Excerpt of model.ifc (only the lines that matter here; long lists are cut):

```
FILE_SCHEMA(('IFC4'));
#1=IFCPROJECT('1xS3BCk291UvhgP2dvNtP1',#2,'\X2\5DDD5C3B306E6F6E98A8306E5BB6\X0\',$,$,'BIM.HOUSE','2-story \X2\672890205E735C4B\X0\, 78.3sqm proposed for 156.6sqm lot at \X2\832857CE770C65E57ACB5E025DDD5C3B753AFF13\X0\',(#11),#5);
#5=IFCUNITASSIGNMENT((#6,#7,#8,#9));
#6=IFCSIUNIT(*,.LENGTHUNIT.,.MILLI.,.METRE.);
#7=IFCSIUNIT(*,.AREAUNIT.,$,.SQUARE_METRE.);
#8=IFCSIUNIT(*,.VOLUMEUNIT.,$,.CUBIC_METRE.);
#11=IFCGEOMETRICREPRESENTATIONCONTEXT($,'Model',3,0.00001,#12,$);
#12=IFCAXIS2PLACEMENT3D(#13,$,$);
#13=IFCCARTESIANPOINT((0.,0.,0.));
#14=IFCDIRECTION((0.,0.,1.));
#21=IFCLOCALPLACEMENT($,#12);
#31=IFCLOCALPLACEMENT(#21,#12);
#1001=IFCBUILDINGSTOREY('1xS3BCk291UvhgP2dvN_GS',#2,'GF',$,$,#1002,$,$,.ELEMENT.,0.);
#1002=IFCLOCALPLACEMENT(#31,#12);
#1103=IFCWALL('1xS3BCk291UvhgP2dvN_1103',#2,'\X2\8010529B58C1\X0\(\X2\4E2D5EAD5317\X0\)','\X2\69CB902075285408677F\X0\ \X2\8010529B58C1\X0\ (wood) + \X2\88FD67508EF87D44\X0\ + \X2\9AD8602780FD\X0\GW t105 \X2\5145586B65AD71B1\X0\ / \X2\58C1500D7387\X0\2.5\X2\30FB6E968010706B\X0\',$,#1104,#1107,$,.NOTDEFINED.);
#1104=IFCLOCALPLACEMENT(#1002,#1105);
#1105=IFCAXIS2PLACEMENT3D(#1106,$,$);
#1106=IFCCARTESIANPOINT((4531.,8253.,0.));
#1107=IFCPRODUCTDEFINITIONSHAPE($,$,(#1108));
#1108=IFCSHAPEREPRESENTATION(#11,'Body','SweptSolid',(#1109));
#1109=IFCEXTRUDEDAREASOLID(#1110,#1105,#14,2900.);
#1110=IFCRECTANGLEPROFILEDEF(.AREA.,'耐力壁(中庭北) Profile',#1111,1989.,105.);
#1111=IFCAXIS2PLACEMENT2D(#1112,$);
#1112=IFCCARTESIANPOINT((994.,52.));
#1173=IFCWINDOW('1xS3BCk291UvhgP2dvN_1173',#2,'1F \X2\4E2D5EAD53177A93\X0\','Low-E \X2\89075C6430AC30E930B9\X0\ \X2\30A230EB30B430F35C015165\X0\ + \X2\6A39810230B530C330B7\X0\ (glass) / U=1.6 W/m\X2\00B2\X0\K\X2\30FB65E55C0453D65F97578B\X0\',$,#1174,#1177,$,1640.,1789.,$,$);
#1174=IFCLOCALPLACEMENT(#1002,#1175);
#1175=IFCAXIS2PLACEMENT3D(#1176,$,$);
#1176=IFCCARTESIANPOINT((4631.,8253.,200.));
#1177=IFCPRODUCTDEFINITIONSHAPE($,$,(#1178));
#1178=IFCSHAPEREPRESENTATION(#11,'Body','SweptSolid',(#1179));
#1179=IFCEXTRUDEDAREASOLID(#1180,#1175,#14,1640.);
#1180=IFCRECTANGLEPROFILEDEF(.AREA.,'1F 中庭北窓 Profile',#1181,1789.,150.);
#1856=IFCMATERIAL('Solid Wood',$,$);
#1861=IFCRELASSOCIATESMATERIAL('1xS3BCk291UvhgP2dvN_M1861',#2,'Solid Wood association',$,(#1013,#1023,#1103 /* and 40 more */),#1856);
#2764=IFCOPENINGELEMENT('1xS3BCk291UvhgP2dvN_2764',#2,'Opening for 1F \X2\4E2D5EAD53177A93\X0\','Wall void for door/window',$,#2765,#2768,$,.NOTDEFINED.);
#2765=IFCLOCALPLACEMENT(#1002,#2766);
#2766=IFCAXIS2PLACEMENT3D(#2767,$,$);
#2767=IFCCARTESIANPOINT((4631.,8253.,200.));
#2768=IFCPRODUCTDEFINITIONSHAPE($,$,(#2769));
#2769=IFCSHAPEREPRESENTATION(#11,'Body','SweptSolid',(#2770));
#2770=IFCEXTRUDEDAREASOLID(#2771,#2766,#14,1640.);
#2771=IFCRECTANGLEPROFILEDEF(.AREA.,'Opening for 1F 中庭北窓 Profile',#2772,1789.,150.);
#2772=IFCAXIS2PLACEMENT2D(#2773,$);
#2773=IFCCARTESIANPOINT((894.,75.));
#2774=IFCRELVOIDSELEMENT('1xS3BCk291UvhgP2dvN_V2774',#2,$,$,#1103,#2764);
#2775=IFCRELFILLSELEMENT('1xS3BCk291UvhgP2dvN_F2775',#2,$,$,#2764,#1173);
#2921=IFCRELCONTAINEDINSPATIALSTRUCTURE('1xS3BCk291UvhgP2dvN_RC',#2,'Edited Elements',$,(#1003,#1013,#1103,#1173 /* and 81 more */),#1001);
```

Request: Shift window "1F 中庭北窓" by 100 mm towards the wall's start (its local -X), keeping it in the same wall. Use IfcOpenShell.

```python
import ifcopenshell
import ifcopenshell.api.geometry
import ifcopenshell.util.placement

model = ifcopenshell.open("model.ifc")

window = model.by_guid("1xS3BCk291UvhgP2dvN_1173")
opening = window.FillsVoids[0].RelatingOpeningElement
wall = opening.VoidsElements[0].RelatingBuildingElement

wall_matrix = ifcopenshell.util.placement.get_local_placement(wall.ObjectPlacement)
shift = wall_matrix[:3, 0] * -100.0
before = ifcopenshell.util.placement.get_local_placement(window.ObjectPlacement)[:3, 3].copy()

# The window is not placed relative to its opening, so move both.
for product in (opening, window):
    matrix = ifcopenshell.util.placement.get_local_placement(product.ObjectPlacement)
    matrix[:3, 3] += shift
    ifcopenshell.api.geometry.edit_object_placement(model, product=product, matrix=matrix, is_si=False)

after = ifcopenshell.util.placement.get_local_placement(window.ObjectPlacement)[:3, 3]
print("window moved by", (after - before).round(3) + 0.0)

model.write("model_edited.ifc")
```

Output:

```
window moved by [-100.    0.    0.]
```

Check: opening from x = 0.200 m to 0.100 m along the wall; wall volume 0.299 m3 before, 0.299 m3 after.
